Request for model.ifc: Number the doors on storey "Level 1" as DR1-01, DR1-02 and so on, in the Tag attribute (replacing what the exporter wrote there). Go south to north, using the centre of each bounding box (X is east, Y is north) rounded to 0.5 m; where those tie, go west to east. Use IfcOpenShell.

First a look at what the model holds.

```python
import ifcopenshell
import ifcopenshell.util.element
import ifcopenshell.util.placement

model = ifcopenshell.open("model.ifc")
print(model.schema)
storey = next(s for s in model.by_type("IfcBuildingStorey") if s.Name == "Level 1")
doors = [e for e in ifcopenshell.util.element.get_decomposition(storey) if e.is_a("IfcDoor")]
for e in sorted(doors, key=lambda e: e.id()):
    origin = ifcopenshell.util.placement.get_local_placement(e.ObjectPlacement)[:3, 3]
    print(e.id(), e.Tag, e.Name, origin.round(2) + 0.0, sep=" | ")
```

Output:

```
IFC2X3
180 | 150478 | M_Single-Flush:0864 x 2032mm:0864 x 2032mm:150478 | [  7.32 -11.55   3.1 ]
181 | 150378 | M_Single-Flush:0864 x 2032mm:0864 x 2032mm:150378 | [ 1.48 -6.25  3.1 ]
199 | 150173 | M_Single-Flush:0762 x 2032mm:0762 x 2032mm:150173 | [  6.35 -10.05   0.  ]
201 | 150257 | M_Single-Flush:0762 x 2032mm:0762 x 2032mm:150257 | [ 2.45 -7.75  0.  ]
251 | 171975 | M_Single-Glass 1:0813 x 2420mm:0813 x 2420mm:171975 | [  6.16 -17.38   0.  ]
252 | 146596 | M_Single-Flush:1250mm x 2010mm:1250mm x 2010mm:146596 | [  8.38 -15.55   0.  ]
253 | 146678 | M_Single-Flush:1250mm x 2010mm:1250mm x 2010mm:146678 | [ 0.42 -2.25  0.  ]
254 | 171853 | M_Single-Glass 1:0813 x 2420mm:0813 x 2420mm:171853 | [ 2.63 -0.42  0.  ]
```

```python
import ifcopenshell
import ifcopenshell.geom
import ifcopenshell.util.element
import ifcopenshell.util.shape

model = ifcopenshell.open("model.ifc")
settings = ifcopenshell.geom.settings()
settings.set("use-world-coords", True)


def centre(element):
    shape = ifcopenshell.geom.create_shape(settings, element)
    return ifcopenshell.util.shape.get_bbox_centroid(shape.geometry)


storey = next(s for s in model.by_type("IfcBuildingStorey") if s.Name == "Level 1")
doors = [e for e in ifcopenshell.util.element.get_decomposition(storey) if e.is_a("IfcDoor")]

# Insertion points can sit at a corner or the storey origin, so sort by the geometry (in metres).
centres = {e: centre(e) for e in doors}
doors.sort(key=lambda e: (round(centres[e][1] / 0.5), centres[e][0]))

for i, e in enumerate(doors, start=1):
    number = f"DR1-{i:02d}"
    e.Tag = number
    print(e.id(), number)

model.write("model_edited.ifc")
```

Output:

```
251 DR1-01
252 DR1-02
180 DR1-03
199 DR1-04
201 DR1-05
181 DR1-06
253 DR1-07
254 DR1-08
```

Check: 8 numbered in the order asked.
